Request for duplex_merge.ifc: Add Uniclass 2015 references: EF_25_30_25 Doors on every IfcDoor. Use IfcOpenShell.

First a look at what the model holds.

```python
import ifcopenshell

model = ifcopenshell.open("duplex_merge.ifc")
print(model.schema)
print("classifications:", [c.Name for c in model.by_type("IfcClassification")])
for ifc_class in ("IfcDoor", "IfcRoof", "IfcStair", "IfcWall", "IfcWindow"):
    print(ifc_class, len(model.by_type(ifc_class)))
```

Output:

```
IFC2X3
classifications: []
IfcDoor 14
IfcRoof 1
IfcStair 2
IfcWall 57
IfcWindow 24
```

```python
import ifcopenshell
import ifcopenshell.api.classification

model = ifcopenshell.open("duplex_merge.ifc")

# IFC2X3 requires Source and Edition and has no link from the project to the system.
system = model.create_entity("IfcClassification", Source="NBS", Edition="2015", Name="Uniclass 2015")

codes = {
    "IfcDoor": ("EF_25_30_25", "Doors"),
}
for ifc_class, (code, name) in codes.items():
    products = model.by_type(ifc_class)
    ifcopenshell.api.classification.add_reference(
        model, products=products, classification=system, identification=code, name=name
    )
    print(code, len(products))

model.write("duplex_merge-out.ifc")
```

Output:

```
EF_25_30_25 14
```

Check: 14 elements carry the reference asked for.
